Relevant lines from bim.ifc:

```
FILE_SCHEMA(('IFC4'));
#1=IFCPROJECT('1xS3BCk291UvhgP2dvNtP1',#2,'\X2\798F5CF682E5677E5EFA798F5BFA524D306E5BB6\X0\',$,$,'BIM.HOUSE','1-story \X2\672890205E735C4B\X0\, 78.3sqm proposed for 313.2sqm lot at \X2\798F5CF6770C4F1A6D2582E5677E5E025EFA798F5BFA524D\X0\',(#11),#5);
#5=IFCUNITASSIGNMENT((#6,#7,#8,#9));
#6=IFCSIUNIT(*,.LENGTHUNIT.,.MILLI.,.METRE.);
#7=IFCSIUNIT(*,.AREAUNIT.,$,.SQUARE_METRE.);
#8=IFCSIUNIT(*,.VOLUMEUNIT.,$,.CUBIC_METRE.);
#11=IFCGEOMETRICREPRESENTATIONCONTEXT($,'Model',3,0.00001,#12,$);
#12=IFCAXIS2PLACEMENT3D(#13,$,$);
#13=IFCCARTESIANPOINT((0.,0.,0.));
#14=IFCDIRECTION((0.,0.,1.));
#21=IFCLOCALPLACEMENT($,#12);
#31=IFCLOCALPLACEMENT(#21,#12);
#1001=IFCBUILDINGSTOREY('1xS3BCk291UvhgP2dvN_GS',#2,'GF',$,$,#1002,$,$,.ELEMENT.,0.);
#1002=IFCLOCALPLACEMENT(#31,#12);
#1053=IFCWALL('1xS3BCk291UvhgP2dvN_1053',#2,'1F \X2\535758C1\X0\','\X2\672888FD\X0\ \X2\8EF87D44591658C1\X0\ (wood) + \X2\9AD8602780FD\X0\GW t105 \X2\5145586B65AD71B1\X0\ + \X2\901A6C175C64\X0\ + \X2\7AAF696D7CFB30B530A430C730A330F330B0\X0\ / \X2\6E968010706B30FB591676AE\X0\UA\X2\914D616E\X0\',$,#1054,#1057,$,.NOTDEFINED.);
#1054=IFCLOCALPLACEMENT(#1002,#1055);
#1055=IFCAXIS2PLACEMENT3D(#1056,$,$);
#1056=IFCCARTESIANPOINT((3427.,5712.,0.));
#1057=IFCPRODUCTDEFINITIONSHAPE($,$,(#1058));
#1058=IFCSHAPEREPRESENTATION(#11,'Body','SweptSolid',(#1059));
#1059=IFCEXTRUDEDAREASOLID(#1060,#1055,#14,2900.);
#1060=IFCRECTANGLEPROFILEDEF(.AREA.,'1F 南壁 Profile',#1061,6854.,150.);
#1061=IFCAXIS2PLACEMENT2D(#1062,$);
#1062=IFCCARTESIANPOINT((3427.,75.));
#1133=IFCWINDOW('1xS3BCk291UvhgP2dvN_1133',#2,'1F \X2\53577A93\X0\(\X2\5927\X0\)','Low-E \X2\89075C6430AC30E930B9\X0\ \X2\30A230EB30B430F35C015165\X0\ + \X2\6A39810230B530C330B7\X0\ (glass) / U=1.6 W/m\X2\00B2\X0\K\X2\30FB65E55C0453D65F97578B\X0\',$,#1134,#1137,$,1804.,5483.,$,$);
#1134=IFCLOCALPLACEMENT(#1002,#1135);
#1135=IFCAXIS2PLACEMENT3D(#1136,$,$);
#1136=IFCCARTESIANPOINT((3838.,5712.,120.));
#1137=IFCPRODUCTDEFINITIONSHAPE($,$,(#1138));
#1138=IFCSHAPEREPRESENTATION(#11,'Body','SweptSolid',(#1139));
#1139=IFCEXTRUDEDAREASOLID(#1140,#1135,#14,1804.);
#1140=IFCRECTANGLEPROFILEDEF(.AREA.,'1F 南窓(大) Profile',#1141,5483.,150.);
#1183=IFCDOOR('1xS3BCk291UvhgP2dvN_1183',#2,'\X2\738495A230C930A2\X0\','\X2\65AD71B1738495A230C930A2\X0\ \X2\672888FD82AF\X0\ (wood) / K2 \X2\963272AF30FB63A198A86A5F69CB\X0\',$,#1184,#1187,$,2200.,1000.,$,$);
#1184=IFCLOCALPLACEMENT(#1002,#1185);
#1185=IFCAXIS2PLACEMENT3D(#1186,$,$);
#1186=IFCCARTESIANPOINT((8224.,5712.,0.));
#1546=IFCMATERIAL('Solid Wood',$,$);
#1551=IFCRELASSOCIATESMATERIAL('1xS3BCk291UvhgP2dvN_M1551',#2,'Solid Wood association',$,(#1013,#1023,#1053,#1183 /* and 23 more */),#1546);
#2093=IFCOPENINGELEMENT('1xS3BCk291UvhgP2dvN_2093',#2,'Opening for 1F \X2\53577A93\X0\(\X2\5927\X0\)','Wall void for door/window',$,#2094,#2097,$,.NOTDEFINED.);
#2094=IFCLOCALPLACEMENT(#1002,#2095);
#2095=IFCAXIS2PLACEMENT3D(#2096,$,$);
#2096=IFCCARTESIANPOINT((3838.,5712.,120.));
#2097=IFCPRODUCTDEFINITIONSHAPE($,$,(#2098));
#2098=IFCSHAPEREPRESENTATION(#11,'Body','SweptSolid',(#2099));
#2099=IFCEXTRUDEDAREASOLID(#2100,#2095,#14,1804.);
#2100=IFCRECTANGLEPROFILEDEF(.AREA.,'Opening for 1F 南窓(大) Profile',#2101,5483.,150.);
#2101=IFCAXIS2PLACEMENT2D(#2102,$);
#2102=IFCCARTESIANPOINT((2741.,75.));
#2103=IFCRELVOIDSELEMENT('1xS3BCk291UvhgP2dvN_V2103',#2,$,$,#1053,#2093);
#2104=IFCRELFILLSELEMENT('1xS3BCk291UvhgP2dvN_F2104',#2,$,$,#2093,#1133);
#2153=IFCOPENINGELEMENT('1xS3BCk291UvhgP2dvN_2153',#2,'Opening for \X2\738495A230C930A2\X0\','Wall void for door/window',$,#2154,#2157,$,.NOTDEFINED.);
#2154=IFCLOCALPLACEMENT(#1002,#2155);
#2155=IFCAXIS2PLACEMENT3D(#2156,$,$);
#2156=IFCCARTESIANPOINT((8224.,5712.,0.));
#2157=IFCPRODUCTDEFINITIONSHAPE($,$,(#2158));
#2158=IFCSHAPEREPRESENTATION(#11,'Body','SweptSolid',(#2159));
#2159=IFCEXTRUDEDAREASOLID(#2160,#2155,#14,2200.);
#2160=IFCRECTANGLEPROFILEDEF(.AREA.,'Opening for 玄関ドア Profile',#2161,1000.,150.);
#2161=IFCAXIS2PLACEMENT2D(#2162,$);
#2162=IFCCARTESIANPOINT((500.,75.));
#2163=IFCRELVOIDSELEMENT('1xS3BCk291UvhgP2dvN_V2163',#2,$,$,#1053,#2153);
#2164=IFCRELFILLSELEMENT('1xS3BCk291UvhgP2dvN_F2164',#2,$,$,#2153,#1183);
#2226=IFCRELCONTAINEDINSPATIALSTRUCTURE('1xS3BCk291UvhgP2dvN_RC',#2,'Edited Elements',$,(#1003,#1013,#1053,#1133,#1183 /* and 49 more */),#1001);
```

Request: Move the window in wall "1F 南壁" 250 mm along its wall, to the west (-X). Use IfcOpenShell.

```python
import ifcopenshell
import ifcopenshell.api.geometry
import ifcopenshell.util.placement
import ifcopenshell.util.unit

model = ifcopenshell.open("bim.ifc")
unit_scale = ifcopenshell.util.unit.calculate_unit_scale(model)

window = model.by_guid("1xS3BCk291UvhgP2dvN_1133")
opening = window.FillsVoids[0].RelatingOpeningElement
wall = opening.VoidsElements[0].RelatingBuildingElement

wall_matrix = ifcopenshell.util.placement.get_local_placement(wall.ObjectPlacement)
shift = wall_matrix[:3, 0] * -0.25 / unit_scale
before = ifcopenshell.util.placement.get_local_placement(window.ObjectPlacement)[:3, 3].copy()

# The window is not placed relative to its opening, so move both.
for product in (opening, window):
    matrix = ifcopenshell.util.placement.get_local_placement(product.ObjectPlacement)
    matrix[:3, 3] += shift
    ifcopenshell.api.geometry.edit_object_placement(model, product=product, matrix=matrix, is_si=False)

after = ifcopenshell.util.placement.get_local_placement(window.ObjectPlacement)[:3, 3]
print("window moved by", (after - before).round(3) + 0.0)

model.write("bim_v2.ifc")
```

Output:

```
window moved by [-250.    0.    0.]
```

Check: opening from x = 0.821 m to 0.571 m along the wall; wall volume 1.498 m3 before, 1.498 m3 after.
